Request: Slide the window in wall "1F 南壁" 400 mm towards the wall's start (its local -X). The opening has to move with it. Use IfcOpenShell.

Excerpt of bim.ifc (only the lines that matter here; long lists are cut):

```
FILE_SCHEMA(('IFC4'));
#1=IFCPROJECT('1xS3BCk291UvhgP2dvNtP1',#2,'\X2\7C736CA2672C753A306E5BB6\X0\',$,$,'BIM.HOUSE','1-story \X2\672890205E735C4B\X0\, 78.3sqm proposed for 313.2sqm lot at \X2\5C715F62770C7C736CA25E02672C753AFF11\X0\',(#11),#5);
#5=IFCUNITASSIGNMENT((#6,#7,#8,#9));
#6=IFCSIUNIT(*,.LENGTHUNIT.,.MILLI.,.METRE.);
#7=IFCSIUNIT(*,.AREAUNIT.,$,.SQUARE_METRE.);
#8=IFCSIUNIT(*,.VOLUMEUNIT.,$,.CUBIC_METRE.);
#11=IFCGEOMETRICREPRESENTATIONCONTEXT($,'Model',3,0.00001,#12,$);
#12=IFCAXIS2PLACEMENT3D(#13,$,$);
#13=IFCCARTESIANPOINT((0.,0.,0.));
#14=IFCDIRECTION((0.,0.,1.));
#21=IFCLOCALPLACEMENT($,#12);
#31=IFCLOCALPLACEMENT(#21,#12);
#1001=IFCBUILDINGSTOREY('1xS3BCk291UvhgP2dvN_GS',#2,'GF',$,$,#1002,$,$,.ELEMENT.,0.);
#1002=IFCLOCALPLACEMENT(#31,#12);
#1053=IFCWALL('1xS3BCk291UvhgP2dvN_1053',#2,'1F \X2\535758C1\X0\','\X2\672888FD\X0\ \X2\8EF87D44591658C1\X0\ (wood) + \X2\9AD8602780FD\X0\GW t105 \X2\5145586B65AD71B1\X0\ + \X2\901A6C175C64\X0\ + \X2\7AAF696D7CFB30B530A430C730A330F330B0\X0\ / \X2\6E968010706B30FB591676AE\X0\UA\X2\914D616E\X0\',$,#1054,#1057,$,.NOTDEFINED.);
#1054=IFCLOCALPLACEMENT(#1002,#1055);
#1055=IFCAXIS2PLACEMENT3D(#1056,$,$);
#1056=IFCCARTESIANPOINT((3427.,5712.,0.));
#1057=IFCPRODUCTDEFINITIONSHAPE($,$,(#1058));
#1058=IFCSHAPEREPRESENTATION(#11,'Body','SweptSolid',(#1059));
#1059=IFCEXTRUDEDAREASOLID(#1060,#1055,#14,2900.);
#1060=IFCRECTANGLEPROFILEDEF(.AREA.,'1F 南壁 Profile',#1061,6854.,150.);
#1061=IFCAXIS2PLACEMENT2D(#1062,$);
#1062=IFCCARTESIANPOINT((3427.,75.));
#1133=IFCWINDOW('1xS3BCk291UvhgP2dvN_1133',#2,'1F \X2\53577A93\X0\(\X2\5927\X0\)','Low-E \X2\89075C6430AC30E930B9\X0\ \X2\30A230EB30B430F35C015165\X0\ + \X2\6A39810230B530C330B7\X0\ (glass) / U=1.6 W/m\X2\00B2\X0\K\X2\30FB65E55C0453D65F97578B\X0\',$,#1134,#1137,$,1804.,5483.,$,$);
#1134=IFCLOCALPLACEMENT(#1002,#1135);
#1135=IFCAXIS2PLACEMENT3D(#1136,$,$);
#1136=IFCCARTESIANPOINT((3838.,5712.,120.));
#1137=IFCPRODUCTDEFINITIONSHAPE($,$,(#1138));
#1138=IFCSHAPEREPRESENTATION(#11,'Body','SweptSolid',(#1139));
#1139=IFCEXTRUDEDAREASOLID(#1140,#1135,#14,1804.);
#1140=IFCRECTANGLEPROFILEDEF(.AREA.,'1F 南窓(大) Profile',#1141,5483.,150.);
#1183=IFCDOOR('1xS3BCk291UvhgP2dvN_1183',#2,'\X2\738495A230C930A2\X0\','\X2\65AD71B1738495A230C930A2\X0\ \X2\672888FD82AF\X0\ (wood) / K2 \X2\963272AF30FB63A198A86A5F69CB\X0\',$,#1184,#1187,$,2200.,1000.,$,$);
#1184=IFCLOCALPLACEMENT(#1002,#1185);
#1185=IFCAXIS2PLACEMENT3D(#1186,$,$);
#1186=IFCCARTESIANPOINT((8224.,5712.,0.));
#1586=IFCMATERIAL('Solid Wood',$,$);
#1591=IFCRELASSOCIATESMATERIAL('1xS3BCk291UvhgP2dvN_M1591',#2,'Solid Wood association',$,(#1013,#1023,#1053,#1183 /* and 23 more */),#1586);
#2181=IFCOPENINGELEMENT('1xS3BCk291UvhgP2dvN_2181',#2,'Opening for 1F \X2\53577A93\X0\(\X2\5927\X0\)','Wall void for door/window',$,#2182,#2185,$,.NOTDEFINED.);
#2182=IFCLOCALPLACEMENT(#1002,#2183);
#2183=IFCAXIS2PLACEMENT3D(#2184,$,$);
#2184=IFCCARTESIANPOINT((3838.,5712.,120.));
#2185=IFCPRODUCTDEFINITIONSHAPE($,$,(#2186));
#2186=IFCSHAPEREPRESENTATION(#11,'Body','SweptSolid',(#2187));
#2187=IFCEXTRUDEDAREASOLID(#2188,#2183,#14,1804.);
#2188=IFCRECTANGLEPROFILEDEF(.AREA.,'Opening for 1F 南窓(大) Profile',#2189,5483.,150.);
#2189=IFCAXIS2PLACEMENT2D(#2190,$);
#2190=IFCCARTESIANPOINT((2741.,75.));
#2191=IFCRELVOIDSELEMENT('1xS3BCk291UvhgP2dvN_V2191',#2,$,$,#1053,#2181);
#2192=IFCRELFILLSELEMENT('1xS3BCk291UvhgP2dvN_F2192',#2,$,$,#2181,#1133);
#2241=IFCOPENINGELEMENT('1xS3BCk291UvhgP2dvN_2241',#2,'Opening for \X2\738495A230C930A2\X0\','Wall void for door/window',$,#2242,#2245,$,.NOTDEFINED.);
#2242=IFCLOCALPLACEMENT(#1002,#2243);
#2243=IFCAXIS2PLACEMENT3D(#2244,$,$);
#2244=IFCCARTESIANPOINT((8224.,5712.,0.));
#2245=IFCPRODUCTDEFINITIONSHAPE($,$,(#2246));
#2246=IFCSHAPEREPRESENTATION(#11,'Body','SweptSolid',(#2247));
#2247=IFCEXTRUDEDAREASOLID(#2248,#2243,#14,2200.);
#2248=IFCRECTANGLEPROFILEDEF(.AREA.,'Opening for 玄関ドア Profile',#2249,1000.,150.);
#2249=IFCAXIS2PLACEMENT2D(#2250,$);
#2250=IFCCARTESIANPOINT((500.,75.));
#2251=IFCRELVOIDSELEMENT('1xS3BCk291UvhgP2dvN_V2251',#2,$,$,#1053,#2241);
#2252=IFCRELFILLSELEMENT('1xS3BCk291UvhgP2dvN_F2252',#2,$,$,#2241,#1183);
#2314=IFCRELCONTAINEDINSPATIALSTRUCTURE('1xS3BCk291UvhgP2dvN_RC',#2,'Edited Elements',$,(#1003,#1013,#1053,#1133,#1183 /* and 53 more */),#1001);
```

```python
import ifcopenshell
import ifcopenshell.api.geometry
import ifcopenshell.util.placement
import ifcopenshell.util.unit

model = ifcopenshell.open("bim.ifc")
unit_scale = ifcopenshell.util.unit.calculate_unit_scale(model)

window = model.by_id(1133)
opening = window.FillsVoids[0].RelatingOpeningElement
wall = opening.VoidsElements[0].RelatingBuildingElement

wall_matrix = ifcopenshell.util.placement.get_local_placement(wall.ObjectPlacement)
shift = wall_matrix[:3, 0] * -0.4 / unit_scale
before = ifcopenshell.util.placement.get_local_placement(window.ObjectPlacement)[:3, 3].copy()

# The window is not placed relative to its opening, so move both.
for product in (opening, window):
    matrix = ifcopenshell.util.placement.get_local_placement(product.ObjectPlacement)
    matrix[:3, 3] += shift
    ifcopenshell.api.geometry.edit_object_placement(model, product=product, matrix=matrix, is_si=False)

after = ifcopenshell.util.placement.get_local_placement(window.ObjectPlacement)[:3, 3]
print("window moved by", (after - before).round(3) + 0.0)

model.write("bim_rev.ifc")
```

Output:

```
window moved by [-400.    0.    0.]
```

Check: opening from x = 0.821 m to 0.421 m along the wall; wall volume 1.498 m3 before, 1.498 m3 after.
